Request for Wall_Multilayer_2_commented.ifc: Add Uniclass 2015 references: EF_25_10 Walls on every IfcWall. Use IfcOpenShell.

First a look at what the model holds.

```python
import ifcopenshell

model = ifcopenshell.open("Wall_Multilayer_2_commented.ifc")
print(model.schema)
print("classifications:", [c.Name for c in model.by_type("IfcClassification")])
for ifc_class in ("IfcDoor", "IfcRoof", "IfcStair", "IfcWall", "IfcWindow"):
    print(ifc_class, len(model.by_type(ifc_class)))
```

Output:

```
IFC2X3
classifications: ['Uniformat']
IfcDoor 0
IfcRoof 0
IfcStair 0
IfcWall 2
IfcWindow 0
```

```python
import ifcopenshell
import ifcopenshell.api.classification

model = ifcopenshell.open("Wall_Multilayer_2_commented.ifc")

# IFC2X3 requires Source and Edition and has no link from the project to the system.
system = model.create_entity("IfcClassification", Source="NBS", Edition="2015", Name="Uniclass 2015")

codes = {
    "IfcWall": ("EF_25_10", "Walls"),
}
for ifc_class, (code, name) in codes.items():
    products = model.by_type(ifc_class)
    ifcopenshell.api.classification.add_reference(
        model, products=products, classification=system, identification=code, name=name
    )
    print(code, len(products))

model.write("Wall_Multilayer_2_commented_v2.ifc")
```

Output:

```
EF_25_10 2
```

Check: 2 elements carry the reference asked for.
